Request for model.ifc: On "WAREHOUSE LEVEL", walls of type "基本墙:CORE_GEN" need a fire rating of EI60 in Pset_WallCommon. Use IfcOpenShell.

First a look at what the model holds.

```python
import ifcopenshell
import ifcopenshell.util.element

model = ifcopenshell.open("model.ifc")
print(model.schema)
storey = next(s for s in model.by_type("IfcBuildingStorey") if s.Name == "WAREHOUSE LEVEL")
walls = [e for e in ifcopenshell.util.element.get_decomposition(storey) if e.is_a("IfcWall")]
seen = {}
for e in walls:
    element_type = ifcopenshell.util.element.get_type(e)
    key = (element_type.Name if element_type != e and element_type else None, ifcopenshell.util.element.get_pset(e, "Pset_WallCommon", "FireRating"))
    seen[key] = seen.get(key, 0) + 1
for (name, value), count in sorted(seen.items(), key=str):
    print(count, "x", name, "|", value)
```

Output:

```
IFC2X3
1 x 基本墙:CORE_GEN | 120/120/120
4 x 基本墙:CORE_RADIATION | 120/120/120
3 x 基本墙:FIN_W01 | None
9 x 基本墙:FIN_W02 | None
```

```python
import ifcopenshell
import ifcopenshell.api.pset
import ifcopenshell.util.element

model = ifcopenshell.open("model.ifc")

storey = next(s for s in model.by_type("IfcBuildingStorey") if s.Name == "WAREHOUSE LEVEL")
walls = [e for e in ifcopenshell.util.element.get_decomposition(storey) if e.is_a("IfcWall")]

count = 0
for e in walls:
    element_type = ifcopenshell.util.element.get_type(e)
    if element_type in (None, e) or element_type.Name != "基本墙:CORE_GEN":
        continue
    # add_pset returns the element's existing set when there is one.
    pset = ifcopenshell.api.pset.add_pset(model, product=e, name="Pset_WallCommon")
    ifcopenshell.api.pset.edit_pset(model, pset=pset, properties={"FireRating": "EI60"})
    count += 1

print(count, "walls updated")

model.write("model_edited.ifc")
```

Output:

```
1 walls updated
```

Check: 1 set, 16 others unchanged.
